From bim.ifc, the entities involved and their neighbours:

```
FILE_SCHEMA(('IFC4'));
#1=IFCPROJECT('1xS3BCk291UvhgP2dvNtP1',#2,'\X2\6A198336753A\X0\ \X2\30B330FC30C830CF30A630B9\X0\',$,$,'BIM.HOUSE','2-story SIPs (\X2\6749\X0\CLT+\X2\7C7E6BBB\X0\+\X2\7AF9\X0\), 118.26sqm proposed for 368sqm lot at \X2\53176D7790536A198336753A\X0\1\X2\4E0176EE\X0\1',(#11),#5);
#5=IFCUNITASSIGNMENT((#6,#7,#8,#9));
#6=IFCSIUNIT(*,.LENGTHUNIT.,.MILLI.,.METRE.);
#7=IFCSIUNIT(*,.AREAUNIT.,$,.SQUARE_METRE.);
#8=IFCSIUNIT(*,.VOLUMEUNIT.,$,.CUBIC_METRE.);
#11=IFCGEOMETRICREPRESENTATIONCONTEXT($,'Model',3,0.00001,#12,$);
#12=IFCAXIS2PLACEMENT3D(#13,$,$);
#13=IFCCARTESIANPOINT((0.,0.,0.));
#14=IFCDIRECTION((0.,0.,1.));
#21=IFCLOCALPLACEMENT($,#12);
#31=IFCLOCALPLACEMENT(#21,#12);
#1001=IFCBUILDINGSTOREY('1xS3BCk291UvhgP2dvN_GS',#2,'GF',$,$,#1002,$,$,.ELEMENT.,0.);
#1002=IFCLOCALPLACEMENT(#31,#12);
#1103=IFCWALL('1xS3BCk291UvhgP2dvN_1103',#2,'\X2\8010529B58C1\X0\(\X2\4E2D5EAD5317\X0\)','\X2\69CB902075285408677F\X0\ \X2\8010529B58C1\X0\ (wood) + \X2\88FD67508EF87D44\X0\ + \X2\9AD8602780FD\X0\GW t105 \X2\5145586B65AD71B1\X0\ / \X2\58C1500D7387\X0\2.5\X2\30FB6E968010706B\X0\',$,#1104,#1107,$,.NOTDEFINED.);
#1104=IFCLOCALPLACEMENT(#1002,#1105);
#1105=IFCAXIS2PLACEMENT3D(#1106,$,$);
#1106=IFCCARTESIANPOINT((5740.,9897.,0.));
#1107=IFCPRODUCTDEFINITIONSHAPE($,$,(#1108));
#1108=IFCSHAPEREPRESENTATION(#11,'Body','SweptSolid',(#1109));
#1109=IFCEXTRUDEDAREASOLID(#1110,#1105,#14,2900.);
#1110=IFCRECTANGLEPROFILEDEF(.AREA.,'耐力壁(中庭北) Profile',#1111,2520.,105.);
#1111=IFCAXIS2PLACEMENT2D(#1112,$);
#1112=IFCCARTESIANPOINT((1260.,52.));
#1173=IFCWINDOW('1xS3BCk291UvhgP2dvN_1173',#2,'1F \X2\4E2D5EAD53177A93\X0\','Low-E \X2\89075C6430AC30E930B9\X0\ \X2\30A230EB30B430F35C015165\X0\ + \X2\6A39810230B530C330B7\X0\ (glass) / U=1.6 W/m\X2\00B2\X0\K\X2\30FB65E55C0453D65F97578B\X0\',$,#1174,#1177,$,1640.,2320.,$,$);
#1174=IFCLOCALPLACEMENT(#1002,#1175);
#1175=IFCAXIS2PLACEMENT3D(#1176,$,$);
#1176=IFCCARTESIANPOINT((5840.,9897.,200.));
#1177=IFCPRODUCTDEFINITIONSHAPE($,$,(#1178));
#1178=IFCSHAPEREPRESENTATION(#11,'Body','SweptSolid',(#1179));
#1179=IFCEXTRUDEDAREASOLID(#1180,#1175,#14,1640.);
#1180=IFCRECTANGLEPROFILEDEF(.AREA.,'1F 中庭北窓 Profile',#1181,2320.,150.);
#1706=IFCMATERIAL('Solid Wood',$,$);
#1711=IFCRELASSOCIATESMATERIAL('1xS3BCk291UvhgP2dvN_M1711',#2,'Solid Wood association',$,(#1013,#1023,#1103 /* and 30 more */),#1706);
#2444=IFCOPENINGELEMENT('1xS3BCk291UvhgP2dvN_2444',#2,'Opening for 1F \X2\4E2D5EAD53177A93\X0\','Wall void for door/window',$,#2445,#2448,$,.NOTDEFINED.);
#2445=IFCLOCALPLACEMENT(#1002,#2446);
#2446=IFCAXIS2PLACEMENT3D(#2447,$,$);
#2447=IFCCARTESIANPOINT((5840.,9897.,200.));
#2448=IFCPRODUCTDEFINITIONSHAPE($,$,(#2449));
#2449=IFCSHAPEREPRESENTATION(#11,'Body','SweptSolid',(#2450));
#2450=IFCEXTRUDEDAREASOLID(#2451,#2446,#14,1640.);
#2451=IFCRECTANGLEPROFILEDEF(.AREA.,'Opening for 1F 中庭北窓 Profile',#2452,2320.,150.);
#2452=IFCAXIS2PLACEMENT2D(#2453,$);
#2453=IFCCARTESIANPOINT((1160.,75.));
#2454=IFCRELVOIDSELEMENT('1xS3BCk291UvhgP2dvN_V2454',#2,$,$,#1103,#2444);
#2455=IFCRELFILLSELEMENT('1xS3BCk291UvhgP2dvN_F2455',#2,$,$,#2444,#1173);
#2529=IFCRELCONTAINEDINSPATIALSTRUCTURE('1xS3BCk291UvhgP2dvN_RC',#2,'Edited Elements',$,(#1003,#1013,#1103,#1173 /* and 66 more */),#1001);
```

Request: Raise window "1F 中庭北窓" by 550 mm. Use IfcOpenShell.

```python
import numpy as np
import ifcopenshell
import ifcopenshell.api.geometry
import ifcopenshell.util.placement
import ifcopenshell.util.unit

model = ifcopenshell.open("bim.ifc")
unit_scale = ifcopenshell.util.unit.calculate_unit_scale(model)

window = model.by_guid("1xS3BCk291UvhgP2dvN_1173")
opening = window.FillsVoids[0].RelatingOpeningElement
dz = 0.55 / unit_scale

shift = np.array([0.0, 0.0, dz])
# The window is not placed relative to its opening, so move both.
for product in (opening, window):
    matrix = ifcopenshell.util.placement.get_local_placement(product.ObjectPlacement)
    matrix[:3, 3] += shift
    ifcopenshell.api.geometry.edit_object_placement(model, product=product, matrix=matrix, is_si=False)

print(f"moved by {dz * unit_scale:+.3f} m")

model.write("bim_updated.ifc")
```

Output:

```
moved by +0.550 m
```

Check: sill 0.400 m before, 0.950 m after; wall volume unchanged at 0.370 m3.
